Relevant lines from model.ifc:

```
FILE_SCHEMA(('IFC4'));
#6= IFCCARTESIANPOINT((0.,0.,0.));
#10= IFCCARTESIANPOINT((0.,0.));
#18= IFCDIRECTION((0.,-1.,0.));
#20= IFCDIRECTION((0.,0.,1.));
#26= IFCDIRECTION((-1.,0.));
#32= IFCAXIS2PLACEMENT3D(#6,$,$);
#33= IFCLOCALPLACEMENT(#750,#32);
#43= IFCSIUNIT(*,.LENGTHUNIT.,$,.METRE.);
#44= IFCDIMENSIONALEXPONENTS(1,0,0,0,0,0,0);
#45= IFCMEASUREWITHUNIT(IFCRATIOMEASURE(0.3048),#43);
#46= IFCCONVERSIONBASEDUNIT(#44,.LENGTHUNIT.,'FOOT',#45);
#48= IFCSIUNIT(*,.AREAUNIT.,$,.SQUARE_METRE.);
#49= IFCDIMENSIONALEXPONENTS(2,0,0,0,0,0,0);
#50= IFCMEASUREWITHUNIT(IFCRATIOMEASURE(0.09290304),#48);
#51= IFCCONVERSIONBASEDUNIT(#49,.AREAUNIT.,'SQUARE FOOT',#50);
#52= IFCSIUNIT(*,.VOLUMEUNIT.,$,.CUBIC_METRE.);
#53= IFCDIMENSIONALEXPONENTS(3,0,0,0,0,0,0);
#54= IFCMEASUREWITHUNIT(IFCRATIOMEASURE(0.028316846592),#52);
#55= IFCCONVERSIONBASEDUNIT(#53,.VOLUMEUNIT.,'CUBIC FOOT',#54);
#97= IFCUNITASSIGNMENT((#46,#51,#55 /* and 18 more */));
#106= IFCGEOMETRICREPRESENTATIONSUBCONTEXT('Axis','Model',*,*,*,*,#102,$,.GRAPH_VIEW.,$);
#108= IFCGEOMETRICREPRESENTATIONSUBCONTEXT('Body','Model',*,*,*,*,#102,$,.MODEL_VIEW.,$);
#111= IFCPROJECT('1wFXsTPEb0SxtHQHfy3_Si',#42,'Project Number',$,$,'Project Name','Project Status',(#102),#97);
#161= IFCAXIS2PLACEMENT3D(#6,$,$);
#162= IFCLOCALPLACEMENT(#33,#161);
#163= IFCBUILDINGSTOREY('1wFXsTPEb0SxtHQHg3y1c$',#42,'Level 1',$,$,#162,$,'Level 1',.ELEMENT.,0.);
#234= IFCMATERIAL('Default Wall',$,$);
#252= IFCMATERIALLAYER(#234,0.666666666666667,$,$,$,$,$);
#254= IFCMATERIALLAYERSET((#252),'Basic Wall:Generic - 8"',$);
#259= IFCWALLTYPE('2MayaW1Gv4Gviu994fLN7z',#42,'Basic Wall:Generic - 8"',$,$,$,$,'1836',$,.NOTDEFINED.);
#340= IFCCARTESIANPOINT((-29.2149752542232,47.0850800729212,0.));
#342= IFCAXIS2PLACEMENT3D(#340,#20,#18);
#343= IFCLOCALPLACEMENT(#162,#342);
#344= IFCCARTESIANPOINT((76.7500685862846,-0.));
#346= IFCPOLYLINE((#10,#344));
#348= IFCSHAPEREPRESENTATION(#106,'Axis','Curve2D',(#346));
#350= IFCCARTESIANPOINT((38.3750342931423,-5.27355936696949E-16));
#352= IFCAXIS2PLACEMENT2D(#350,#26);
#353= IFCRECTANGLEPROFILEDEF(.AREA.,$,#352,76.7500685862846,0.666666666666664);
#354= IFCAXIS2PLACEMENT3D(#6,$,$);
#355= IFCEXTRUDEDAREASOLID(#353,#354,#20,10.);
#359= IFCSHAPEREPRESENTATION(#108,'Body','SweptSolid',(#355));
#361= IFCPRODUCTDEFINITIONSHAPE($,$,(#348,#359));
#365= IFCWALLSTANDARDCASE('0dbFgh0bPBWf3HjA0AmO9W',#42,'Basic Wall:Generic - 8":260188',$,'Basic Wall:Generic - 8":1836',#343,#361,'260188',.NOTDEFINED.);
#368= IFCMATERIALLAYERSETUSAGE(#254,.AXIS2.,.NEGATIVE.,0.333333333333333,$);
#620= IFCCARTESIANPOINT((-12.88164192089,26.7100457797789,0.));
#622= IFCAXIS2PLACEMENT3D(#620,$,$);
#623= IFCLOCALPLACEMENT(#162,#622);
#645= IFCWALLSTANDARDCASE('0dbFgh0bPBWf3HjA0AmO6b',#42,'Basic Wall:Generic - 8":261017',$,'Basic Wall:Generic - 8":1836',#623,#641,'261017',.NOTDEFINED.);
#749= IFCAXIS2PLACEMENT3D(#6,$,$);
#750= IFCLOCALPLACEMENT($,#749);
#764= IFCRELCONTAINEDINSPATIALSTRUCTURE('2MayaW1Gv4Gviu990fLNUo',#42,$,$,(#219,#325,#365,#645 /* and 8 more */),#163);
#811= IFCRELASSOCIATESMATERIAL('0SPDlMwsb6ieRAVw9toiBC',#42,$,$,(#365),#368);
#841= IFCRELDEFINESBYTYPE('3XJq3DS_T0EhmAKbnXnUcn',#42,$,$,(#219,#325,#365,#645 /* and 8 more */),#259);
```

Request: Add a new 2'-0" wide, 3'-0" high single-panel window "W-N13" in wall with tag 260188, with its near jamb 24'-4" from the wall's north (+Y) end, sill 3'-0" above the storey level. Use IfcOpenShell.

```python
import numpy as np
import ifcopenshell
import ifcopenshell.api.feature
import ifcopenshell.api.geometry
import ifcopenshell.api.root
import ifcopenshell.api.spatial
import ifcopenshell.geom
import ifcopenshell.util.element
import ifcopenshell.util.placement
import ifcopenshell.util.representation
import ifcopenshell.util.shape
import ifcopenshell.util.unit

model = ifcopenshell.open("model.ifc")
unit_scale = ifcopenshell.util.unit.calculate_unit_scale(model)
settings = ifcopenshell.geom.settings()


def volume(element):
    """Net volume in cubic metres, openings subtracted."""
    shape = ifcopenshell.geom.create_shape(settings, element)
    return ifcopenshell.util.shape.get_volume(shape.geometry)


wall = model.by_guid("0dbFgh0bPBWf3HjA0AmO9W")
storey = ifcopenshell.util.element.get_container(wall, ifc_class="IfcBuildingStorey")
context = ifcopenshell.util.representation.get_context(model, "Model", "Body", "MODEL_VIEW")
before = volume(wall)

width, height, from_end, sill = 0.6096, 0.9144, 7.4168, 0.9144  # metres

# The wall runs along its own X axis, and the end named is its -X end.
wall_shape = ifcopenshell.geom.create_shape(settings, wall)
x, y, z = ifcopenshell.util.shape.get_vertices(wall_shape.geometry).T
start = x.min() + from_end
face, thickness = float(y.min()), float(y.max() - y.min())
wall_matrix = ifcopenshell.util.placement.get_local_placement(wall.ObjectPlacement)
level = ifcopenshell.util.placement.get_local_placement(storey.ObjectPlacement)[2, 3]


def in_wall(x, y):
    """Placement at x, y metres in the wall's axes, at sill height."""
    matrix = wall_matrix.copy()
    matrix[:, 3] = wall_matrix @ np.array([x / unit_scale, y / unit_scale, 0.0, 1.0])
    matrix[2, 3] = level + sill / unit_scale
    return matrix


# Opening: a box that overshoots both wall faces by 50 mm.
opening = ifcopenshell.api.root.create_entity(model, ifc_class="IfcOpeningElement", predefined_type="OPENING")
box = ifcopenshell.api.geometry.add_wall_representation(
    model, context=context, length=width, height=height, thickness=thickness + 0.1
)
ifcopenshell.api.geometry.assign_representation(model, product=opening, representation=box)
ifcopenshell.api.geometry.edit_object_placement(model, product=opening, matrix=in_wall(start, face - 0.05), is_si=False)
ifcopenshell.api.feature.add_feature(model, feature=opening, element=wall)

window = ifcopenshell.api.root.create_entity(model, ifc_class="IfcWindow", name="W-N13", predefined_type="WINDOW")
window.OverallWidth, window.OverallHeight = width / unit_scale, height / unit_scale
window.PartitioningType = "SINGLE_PANEL"
body = ifcopenshell.api.geometry.add_window_representation(
    model,
    context=context,
    overall_width=window.OverallWidth,
    overall_height=window.OverallHeight,
    partition_type="SINGLE_PANEL",
)
ifcopenshell.api.geometry.assign_representation(model, product=window, representation=body)
ifcopenshell.api.spatial.assign_container(model, products=[window], relating_structure=storey)
ifcopenshell.api.feature.add_filling(model, opening=opening, element=window)

# Centre the window in the wall's thickness.
ifcopenshell.api.geometry.edit_object_placement(model, product=window, matrix=in_wall(start, face), is_si=False)
window_shape = ifcopenshell.geom.create_shape(settings, window)
depth = ifcopenshell.util.shape.get_vertices(window_shape.geometry)[:, 1]
offset = face + thickness / 2 - (depth.min() + depth.max()) / 2
ifcopenshell.api.geometry.edit_object_placement(model, product=window, matrix=in_wall(start, offset), is_si=False)

after = volume(wall)

print(f"wall volume {before:.3f} -> {after:.3f} m3")

model.write("model-out.ifc")
```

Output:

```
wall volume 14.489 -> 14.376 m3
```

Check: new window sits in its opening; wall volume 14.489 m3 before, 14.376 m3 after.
